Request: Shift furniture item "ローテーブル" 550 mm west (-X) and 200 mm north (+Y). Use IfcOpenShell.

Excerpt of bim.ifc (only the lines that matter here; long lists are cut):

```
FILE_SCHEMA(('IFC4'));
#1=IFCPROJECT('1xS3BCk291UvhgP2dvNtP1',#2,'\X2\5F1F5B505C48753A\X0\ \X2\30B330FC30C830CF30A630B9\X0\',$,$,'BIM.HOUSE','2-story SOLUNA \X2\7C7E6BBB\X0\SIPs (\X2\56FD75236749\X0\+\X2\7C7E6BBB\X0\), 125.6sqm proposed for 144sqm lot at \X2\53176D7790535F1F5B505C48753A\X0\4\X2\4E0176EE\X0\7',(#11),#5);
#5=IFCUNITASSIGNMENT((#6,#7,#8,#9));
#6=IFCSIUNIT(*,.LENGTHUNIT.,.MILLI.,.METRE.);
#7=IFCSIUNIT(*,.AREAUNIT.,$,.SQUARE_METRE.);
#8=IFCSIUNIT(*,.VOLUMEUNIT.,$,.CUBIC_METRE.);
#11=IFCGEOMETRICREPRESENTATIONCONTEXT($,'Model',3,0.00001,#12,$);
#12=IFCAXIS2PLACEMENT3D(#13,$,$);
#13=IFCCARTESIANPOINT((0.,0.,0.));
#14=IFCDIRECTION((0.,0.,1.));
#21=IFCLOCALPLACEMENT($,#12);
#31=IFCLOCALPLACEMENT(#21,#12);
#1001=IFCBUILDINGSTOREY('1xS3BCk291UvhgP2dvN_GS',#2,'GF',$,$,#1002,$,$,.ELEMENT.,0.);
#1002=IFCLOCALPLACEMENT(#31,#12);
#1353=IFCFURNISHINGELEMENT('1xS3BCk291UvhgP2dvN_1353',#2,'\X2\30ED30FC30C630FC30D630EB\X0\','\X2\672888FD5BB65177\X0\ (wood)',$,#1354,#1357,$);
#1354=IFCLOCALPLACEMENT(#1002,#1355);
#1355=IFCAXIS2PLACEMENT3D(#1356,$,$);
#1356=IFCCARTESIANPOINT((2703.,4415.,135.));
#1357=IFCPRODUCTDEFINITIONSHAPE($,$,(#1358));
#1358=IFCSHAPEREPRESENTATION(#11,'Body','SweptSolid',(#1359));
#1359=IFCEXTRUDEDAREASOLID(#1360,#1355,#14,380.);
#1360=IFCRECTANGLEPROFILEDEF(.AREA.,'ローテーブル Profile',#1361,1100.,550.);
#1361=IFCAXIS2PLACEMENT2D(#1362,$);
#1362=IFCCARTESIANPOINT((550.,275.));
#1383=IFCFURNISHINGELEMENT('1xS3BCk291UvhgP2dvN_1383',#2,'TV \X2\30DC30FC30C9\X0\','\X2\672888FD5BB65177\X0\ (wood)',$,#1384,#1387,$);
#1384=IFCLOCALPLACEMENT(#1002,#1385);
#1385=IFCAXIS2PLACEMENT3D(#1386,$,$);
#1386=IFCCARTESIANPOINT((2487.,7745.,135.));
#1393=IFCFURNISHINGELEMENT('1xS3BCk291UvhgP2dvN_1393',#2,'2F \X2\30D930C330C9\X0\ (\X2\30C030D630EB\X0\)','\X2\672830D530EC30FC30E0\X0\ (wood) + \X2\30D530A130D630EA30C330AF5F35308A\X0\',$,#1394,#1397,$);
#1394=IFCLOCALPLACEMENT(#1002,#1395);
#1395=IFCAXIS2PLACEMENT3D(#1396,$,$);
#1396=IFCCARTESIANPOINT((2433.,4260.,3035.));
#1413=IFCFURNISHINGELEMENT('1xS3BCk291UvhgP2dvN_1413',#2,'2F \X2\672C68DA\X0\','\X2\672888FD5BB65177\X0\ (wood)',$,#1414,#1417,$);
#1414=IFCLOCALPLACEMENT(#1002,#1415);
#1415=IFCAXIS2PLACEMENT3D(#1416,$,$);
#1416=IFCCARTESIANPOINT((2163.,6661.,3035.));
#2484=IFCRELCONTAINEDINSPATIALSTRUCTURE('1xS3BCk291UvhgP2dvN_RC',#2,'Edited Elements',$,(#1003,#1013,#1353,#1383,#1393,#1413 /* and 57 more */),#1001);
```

```python
import ifcopenshell
import ifcopenshell.api.geometry
import ifcopenshell.util.placement
import ifcopenshell.util.unit

model = ifcopenshell.open("bim.ifc")
unit_scale = ifcopenshell.util.unit.calculate_unit_scale(model)

item = model.by_guid("1xS3BCk291UvhgP2dvN_1353")
matrix = ifcopenshell.util.placement.get_local_placement(item.ObjectPlacement)
matrix[0, 3] -= 0.55 / unit_scale
matrix[1, 3] += 0.2 / unit_scale
ifcopenshell.api.geometry.edit_object_placement(model, product=item, matrix=matrix, is_si=False)

print(ifcopenshell.util.placement.get_local_placement(item.ObjectPlacement).round(3) + 0.0)

model.write("bim_rev.ifc")
```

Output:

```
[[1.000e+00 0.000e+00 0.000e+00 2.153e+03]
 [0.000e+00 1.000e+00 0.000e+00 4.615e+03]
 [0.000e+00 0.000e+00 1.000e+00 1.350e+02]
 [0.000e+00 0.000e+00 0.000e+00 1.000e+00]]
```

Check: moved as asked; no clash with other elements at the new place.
